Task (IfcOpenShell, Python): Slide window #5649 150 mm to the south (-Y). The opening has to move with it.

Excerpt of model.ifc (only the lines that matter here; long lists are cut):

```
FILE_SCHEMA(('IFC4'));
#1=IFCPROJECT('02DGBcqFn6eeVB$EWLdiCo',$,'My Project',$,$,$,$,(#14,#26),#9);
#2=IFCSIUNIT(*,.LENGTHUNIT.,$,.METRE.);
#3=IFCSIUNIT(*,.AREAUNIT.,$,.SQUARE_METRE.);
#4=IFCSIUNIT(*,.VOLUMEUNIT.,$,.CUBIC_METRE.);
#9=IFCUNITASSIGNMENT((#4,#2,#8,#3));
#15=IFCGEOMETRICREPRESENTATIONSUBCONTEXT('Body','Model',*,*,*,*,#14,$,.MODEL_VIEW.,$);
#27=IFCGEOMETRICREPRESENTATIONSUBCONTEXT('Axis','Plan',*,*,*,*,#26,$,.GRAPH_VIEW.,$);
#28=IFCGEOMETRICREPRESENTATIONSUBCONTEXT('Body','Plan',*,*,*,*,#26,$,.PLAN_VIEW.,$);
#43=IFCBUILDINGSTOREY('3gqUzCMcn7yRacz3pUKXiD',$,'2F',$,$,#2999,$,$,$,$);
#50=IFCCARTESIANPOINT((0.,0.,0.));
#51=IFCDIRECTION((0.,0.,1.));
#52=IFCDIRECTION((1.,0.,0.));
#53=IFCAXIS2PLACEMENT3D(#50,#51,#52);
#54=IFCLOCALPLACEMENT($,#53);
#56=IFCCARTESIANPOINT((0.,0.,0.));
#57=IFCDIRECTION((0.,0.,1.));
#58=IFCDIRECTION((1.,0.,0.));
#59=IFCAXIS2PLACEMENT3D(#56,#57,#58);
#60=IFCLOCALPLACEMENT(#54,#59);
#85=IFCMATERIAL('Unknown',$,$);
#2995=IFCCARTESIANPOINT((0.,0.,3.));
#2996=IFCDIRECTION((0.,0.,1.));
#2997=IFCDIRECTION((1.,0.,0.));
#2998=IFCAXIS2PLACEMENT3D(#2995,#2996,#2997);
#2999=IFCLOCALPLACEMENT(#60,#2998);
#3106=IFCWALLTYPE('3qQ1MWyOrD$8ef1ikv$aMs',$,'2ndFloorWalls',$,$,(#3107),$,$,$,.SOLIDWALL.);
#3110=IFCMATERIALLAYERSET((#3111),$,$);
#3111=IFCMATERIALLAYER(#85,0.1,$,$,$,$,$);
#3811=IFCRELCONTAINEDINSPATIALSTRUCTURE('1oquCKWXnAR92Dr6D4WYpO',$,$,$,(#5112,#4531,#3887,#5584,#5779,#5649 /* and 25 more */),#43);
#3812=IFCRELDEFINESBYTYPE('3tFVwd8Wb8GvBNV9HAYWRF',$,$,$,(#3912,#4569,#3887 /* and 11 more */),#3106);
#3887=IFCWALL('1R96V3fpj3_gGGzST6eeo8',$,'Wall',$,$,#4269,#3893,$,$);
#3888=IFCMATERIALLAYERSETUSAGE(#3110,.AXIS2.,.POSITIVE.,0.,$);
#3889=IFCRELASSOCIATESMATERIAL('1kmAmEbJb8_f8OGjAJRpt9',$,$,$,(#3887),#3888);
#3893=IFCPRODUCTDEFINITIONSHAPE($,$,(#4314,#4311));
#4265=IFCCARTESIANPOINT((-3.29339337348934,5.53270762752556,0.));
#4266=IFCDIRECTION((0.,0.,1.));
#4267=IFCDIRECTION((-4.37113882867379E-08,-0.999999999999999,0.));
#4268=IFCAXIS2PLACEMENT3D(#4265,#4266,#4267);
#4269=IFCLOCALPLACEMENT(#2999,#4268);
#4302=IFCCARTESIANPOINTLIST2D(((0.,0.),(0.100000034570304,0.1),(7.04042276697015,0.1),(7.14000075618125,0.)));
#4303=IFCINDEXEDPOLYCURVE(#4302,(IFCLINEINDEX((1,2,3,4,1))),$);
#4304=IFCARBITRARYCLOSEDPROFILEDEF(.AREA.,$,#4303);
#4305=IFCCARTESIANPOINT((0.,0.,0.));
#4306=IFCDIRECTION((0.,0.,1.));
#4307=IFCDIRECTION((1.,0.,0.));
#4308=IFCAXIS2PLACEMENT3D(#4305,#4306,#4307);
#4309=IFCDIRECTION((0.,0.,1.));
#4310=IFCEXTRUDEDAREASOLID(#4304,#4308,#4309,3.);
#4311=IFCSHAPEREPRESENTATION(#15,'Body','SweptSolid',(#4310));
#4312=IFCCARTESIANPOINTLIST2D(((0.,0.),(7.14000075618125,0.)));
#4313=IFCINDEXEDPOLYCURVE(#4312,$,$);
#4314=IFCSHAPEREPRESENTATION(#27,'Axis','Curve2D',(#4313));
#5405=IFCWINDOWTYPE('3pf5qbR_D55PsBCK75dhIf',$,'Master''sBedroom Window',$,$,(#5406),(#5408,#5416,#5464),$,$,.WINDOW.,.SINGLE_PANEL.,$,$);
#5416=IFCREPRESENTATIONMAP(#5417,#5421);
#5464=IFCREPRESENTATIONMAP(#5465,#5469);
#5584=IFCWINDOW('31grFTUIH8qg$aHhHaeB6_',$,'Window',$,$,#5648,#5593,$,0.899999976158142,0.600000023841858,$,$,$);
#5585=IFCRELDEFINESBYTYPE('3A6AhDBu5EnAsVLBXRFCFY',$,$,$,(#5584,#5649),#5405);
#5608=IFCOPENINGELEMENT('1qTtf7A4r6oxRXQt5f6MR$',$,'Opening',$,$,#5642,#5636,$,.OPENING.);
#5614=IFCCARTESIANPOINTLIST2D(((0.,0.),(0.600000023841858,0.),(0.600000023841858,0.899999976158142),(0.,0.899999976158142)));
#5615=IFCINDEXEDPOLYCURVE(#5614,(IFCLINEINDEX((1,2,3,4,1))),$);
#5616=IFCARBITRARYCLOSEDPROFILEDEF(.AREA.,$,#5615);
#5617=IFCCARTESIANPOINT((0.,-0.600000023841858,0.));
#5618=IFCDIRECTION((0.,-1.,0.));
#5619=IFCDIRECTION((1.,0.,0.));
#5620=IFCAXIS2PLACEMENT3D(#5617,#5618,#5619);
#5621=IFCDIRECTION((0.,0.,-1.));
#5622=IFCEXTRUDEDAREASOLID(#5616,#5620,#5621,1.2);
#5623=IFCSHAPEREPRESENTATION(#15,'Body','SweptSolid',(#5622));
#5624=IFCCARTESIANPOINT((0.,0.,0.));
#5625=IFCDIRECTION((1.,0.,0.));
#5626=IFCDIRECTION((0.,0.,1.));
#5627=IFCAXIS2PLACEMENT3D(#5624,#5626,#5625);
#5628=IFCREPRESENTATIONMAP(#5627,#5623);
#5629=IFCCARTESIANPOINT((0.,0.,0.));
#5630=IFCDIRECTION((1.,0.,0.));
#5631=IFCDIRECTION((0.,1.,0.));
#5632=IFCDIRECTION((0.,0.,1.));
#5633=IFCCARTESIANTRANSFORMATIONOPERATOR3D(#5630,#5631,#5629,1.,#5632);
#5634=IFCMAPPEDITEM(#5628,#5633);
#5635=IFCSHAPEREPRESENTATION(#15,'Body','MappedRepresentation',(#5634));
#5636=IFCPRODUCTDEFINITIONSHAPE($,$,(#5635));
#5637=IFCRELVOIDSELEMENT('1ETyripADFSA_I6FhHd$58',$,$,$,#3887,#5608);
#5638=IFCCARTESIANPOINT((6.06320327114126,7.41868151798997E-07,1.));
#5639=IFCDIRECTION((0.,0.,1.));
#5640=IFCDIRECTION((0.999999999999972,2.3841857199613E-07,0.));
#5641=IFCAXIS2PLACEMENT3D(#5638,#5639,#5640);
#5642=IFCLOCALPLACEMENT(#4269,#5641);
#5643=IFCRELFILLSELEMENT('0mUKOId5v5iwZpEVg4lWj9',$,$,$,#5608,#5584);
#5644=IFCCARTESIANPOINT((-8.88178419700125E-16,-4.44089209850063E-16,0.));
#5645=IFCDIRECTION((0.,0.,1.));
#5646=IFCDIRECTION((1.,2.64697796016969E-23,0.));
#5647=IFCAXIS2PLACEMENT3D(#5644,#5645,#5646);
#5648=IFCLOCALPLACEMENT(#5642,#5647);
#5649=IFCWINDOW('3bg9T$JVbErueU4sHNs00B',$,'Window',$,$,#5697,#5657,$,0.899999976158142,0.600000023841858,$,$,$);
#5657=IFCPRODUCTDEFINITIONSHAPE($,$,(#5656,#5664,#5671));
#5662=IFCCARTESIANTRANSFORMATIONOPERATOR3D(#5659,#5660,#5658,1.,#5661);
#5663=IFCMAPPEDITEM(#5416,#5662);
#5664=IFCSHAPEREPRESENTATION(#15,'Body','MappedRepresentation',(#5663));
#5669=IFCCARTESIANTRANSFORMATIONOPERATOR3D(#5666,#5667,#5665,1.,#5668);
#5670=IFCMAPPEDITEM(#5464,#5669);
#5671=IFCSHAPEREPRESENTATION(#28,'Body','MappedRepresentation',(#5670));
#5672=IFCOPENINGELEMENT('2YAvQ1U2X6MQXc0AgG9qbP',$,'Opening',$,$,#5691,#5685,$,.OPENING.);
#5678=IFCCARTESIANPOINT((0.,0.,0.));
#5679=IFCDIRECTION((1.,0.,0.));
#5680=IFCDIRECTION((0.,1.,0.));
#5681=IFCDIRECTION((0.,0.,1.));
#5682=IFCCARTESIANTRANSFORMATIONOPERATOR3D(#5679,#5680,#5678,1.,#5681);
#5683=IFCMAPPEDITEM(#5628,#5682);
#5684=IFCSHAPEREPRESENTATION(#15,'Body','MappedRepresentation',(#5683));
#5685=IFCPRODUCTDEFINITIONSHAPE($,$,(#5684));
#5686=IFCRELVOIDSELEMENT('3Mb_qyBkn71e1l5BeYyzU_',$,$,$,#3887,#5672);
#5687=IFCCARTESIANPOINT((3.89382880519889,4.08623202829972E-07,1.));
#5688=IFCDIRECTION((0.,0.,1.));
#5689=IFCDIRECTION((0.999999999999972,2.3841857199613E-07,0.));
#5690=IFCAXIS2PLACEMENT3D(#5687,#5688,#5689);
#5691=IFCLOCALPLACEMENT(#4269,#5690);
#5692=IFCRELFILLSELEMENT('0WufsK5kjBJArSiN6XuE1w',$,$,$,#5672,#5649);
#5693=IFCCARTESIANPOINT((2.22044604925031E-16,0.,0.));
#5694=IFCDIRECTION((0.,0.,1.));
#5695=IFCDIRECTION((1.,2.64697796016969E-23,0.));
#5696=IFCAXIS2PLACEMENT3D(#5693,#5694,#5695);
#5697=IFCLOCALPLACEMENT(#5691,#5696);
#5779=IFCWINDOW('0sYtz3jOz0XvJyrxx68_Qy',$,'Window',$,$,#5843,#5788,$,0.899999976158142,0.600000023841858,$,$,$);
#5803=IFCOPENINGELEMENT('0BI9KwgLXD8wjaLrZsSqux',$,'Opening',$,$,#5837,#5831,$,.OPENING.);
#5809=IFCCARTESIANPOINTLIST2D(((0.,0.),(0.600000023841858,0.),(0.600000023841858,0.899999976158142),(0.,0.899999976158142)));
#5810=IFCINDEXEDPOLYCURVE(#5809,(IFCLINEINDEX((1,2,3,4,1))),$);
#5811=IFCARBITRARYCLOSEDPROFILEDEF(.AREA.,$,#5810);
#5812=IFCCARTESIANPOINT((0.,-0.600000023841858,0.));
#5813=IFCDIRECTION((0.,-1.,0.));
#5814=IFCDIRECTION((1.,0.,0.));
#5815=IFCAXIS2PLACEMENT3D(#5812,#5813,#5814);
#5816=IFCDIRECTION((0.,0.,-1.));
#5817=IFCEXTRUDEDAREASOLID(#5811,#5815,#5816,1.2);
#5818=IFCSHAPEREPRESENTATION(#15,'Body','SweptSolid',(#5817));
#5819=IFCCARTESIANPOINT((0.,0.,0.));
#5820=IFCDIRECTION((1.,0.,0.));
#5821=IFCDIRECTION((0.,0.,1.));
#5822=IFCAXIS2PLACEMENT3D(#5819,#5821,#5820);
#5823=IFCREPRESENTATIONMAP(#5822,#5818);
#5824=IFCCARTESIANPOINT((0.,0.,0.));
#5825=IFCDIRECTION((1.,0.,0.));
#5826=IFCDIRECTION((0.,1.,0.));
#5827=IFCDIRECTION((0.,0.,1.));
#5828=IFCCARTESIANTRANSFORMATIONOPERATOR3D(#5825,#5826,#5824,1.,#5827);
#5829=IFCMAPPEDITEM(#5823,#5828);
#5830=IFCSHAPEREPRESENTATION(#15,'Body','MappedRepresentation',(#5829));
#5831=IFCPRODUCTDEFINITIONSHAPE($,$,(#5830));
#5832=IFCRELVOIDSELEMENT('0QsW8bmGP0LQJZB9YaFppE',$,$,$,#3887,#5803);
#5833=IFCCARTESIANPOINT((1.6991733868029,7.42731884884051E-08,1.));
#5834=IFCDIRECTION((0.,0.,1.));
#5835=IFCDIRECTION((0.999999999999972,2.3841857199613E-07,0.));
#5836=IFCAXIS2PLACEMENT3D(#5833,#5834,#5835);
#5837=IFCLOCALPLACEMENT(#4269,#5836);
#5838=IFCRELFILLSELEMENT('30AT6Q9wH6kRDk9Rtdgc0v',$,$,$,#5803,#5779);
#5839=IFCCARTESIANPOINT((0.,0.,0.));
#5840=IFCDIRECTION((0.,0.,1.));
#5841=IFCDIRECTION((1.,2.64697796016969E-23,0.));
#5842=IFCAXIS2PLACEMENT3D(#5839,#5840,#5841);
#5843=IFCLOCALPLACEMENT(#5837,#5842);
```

```python
import ifcopenshell
import ifcopenshell.api.geometry
import ifcopenshell.util.placement
import ifcopenshell.util.unit

model = ifcopenshell.open("model.ifc")
unit_scale = ifcopenshell.util.unit.calculate_unit_scale(model)

window = model.by_id(5649)
opening = window.FillsVoids[0].RelatingOpeningElement
wall = opening.VoidsElements[0].RelatingBuildingElement

wall_matrix = ifcopenshell.util.placement.get_local_placement(wall.ObjectPlacement)
shift = wall_matrix[:3, 0] * 0.15 / unit_scale
before = ifcopenshell.util.placement.get_local_placement(window.ObjectPlacement)[:3, 3].copy()

# The window is placed relative to its opening, so it follows when the opening moves.
matrix = ifcopenshell.util.placement.get_local_placement(opening.ObjectPlacement)
matrix[:3, 3] += shift
ifcopenshell.api.geometry.edit_object_placement(
    model, product=opening, matrix=matrix, is_si=False, should_transform_children=True
)

after = ifcopenshell.util.placement.get_local_placement(window.ObjectPlacement)[:3, 3]
print("window moved by", (after - before).round(3) + 0.0)

model.write("model_edited.ifc")
```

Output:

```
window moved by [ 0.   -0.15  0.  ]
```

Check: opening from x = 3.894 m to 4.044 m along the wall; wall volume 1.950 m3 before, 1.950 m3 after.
